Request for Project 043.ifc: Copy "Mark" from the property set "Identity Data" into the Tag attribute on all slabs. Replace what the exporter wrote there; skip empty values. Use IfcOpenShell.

First a look at what the model holds.

```python
import ifcopenshell
import ifcopenshell.util.element

model = ifcopenshell.open("Project 043.ifc")
print(model.schema)
slabs = model.by_type("IfcSlab")
print(len(slabs), "slabs")
for e in slabs[:8]:
    source = ifcopenshell.util.element.get_pset(e, "Identity Data", "Mark")
    target = e.Tag
    print(e.id(), repr(source), repr(target), sep=" | ")
```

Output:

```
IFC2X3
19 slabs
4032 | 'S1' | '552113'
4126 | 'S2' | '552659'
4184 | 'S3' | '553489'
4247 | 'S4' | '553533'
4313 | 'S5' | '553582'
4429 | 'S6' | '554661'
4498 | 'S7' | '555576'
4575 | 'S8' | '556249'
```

```python
import ifcopenshell
import ifcopenshell.util.element

model = ifcopenshell.open("Project 043.ifc")

count = 0
for e in model.by_type("IfcSlab"):
    value = ifcopenshell.util.element.get_pset(e, "Identity Data", "Mark")
    current = e.Tag
    if not value or not value.strip() or current == value:
        continue
    e.Tag = value
    count += 1

print(count, "slabs updated")

model.write("Project 043_rev.ifc")
```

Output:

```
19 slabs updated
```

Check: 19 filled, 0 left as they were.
